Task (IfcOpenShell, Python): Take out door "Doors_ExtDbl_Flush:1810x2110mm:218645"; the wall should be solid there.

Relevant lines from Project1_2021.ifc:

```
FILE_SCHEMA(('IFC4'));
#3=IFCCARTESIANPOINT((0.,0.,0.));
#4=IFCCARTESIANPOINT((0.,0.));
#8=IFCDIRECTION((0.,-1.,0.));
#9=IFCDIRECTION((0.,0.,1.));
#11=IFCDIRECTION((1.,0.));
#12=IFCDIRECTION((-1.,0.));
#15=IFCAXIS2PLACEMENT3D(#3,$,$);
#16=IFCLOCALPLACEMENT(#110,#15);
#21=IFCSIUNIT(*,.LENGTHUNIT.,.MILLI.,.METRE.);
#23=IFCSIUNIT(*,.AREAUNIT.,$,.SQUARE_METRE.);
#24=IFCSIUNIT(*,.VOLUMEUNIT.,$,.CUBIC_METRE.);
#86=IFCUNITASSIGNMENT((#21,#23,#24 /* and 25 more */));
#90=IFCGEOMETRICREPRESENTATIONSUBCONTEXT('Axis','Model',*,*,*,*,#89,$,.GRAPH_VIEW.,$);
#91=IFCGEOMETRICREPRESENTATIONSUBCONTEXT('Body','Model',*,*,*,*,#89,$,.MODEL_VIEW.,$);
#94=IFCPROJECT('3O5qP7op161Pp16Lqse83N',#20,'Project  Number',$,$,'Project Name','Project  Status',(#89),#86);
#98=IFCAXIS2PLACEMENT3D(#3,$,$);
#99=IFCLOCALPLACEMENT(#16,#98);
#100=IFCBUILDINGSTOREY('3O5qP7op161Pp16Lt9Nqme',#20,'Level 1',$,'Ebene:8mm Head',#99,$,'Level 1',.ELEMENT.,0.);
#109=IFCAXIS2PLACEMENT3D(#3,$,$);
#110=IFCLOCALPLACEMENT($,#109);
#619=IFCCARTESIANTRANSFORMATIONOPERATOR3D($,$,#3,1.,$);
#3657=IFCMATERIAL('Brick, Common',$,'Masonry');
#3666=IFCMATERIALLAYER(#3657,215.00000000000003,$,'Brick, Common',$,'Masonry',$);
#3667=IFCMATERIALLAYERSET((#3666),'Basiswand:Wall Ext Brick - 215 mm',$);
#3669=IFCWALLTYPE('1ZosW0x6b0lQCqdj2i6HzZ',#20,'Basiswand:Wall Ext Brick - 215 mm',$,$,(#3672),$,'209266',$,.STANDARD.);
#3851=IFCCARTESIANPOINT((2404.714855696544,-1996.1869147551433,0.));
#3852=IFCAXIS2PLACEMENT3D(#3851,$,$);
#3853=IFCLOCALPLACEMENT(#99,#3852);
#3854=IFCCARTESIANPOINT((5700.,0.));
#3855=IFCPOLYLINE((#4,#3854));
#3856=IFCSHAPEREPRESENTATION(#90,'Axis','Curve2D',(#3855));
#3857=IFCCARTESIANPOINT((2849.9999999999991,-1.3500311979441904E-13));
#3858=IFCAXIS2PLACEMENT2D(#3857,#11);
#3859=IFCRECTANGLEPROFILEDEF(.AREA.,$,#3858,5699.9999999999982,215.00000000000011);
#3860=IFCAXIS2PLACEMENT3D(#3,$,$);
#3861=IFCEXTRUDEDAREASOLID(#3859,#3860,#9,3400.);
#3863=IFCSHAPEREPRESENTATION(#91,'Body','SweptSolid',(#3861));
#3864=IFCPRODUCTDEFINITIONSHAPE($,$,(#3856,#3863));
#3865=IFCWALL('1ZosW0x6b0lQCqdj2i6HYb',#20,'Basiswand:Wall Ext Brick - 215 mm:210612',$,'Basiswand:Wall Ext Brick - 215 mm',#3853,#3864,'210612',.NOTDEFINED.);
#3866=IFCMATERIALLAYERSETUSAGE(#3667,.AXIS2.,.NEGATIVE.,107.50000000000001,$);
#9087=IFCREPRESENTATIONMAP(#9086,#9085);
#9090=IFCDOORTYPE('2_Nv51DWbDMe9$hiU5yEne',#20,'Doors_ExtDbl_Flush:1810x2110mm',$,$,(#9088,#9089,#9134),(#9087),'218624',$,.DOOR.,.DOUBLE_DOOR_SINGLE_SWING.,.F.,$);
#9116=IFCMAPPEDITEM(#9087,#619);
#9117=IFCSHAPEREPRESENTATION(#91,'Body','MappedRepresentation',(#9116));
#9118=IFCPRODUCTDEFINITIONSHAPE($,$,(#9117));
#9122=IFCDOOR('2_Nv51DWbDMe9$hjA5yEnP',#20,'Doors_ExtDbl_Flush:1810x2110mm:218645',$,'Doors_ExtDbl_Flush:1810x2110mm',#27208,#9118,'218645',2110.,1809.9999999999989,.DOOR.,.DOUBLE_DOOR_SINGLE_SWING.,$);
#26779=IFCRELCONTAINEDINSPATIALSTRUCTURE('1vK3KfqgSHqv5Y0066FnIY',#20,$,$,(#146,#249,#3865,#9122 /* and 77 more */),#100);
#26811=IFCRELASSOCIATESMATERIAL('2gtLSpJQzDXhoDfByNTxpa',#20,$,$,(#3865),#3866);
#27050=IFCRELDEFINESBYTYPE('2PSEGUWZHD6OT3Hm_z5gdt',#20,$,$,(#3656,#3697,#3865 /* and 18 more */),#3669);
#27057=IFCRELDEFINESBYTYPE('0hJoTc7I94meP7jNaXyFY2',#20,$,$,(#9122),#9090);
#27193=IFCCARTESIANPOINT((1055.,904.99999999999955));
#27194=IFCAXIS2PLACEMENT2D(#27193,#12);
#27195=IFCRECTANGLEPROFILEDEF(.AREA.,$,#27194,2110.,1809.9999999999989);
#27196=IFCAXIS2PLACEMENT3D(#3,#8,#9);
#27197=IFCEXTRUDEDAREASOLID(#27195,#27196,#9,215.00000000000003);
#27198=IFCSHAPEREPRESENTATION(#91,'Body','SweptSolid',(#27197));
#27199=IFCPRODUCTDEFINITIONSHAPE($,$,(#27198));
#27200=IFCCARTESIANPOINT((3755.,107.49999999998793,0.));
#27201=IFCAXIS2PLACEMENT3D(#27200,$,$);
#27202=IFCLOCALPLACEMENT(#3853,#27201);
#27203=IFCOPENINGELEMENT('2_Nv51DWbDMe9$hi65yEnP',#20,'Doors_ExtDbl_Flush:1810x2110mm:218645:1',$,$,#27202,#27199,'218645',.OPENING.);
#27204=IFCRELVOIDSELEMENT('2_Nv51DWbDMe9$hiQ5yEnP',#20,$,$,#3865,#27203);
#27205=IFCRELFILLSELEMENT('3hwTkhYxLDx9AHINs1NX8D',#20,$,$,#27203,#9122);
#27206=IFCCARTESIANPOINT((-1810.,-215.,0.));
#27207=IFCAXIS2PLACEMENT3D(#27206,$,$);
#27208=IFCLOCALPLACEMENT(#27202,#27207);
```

```python
import ifcopenshell
import ifcopenshell.api.feature
import ifcopenshell.api.root
import ifcopenshell.geom
import ifcopenshell.util.shape

model = ifcopenshell.open("Project1_2021.ifc")
settings = ifcopenshell.geom.settings()


def volume(element):
    """Net volume in cubic metres, openings subtracted."""
    shape = ifcopenshell.geom.create_shape(settings, element)
    return ifcopenshell.util.shape.get_volume(shape.geometry)


door = model.by_guid("2_Nv51DWbDMe9$hjA5yEnP")
opening = door.FillsVoids[0].RelatingOpeningElement
wall = opening.VoidsElements[0].RelatingBuildingElement
before = volume(wall)

ifcopenshell.api.root.remove_product(model, product=door)
ifcopenshell.api.feature.remove_feature(model, feature=opening)

after = volume(wall)

print(f"wall volume {before:.3f} -> {after:.3f} m3")

model.write("Project1_2021_edited.ifc")
```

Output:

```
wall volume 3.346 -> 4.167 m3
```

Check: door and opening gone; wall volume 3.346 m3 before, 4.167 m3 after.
